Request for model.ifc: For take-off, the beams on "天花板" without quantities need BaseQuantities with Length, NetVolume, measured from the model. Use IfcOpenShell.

First a look at what the model holds.

```python
import ifcopenshell
import ifcopenshell.util.element
import ifcopenshell.util.unit

model = ifcopenshell.open("model.ifc")
print(model.schema)
for unit_type in ("LENGTHUNIT", "AREAUNIT", "VOLUMEUNIT"):
    print(unit_type, ifcopenshell.util.unit.calculate_unit_scale(model, unit_type))
storey = next(s for s in model.by_type("IfcBuildingStorey") if s.Name == "天花板")
beams = [e for e in ifcopenshell.util.element.get_decomposition(storey) if e.is_a("IfcBeam")]
for e in sorted(beams, key=lambda e: e.id()):
    print(e.id(), e.is_a(), e.Name, list(ifcopenshell.util.element.get_psets(e, qtos_only=True)), sep=" | ")
```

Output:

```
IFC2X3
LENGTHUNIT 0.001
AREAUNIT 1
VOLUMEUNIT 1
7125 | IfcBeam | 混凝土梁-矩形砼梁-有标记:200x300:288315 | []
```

```python
import ifcopenshell
import ifcopenshell.api.pset
import ifcopenshell.geom
import ifcopenshell.util.element
import ifcopenshell.util.shape
import ifcopenshell.util.unit

model = ifcopenshell.open("model.ifc")
unit_scale = ifcopenshell.util.unit.calculate_unit_scale(model)
volume_scale = ifcopenshell.util.unit.calculate_unit_scale(model, "VOLUMEUNIT")
settings = ifcopenshell.geom.settings()

storey = next(s for s in model.by_type("IfcBuildingStorey") if s.Name == "天花板")
beams = [e for e in ifcopenshell.util.element.get_decomposition(storey) if e.is_a("IfcBeam")]

for e in sorted(beams, key=lambda e: e.id()):
    if ifcopenshell.util.element.get_psets(e, qtos_only=True, should_inherit=False):
        continue
    # Geometry comes back in metres, in the element's own axes.
    shape = ifcopenshell.geom.create_shape(settings, e)
    values = {
        "Length": ifcopenshell.util.shape.get_max_xyz(shape.geometry) / unit_scale,
        "NetVolume": ifcopenshell.util.shape.get_volume(shape.geometry) / volume_scale,
    }
    qto = ifcopenshell.api.pset.add_qto(model, product=e, name="BaseQuantities")
    ifcopenshell.api.pset.edit_qto(model, qto=qto, properties=values)
    print(e.id(), {k: round(v, 3) for k, v in values.items()})

model.write("model_rev.ifc")
```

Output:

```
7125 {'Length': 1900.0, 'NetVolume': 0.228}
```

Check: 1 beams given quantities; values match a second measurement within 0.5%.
